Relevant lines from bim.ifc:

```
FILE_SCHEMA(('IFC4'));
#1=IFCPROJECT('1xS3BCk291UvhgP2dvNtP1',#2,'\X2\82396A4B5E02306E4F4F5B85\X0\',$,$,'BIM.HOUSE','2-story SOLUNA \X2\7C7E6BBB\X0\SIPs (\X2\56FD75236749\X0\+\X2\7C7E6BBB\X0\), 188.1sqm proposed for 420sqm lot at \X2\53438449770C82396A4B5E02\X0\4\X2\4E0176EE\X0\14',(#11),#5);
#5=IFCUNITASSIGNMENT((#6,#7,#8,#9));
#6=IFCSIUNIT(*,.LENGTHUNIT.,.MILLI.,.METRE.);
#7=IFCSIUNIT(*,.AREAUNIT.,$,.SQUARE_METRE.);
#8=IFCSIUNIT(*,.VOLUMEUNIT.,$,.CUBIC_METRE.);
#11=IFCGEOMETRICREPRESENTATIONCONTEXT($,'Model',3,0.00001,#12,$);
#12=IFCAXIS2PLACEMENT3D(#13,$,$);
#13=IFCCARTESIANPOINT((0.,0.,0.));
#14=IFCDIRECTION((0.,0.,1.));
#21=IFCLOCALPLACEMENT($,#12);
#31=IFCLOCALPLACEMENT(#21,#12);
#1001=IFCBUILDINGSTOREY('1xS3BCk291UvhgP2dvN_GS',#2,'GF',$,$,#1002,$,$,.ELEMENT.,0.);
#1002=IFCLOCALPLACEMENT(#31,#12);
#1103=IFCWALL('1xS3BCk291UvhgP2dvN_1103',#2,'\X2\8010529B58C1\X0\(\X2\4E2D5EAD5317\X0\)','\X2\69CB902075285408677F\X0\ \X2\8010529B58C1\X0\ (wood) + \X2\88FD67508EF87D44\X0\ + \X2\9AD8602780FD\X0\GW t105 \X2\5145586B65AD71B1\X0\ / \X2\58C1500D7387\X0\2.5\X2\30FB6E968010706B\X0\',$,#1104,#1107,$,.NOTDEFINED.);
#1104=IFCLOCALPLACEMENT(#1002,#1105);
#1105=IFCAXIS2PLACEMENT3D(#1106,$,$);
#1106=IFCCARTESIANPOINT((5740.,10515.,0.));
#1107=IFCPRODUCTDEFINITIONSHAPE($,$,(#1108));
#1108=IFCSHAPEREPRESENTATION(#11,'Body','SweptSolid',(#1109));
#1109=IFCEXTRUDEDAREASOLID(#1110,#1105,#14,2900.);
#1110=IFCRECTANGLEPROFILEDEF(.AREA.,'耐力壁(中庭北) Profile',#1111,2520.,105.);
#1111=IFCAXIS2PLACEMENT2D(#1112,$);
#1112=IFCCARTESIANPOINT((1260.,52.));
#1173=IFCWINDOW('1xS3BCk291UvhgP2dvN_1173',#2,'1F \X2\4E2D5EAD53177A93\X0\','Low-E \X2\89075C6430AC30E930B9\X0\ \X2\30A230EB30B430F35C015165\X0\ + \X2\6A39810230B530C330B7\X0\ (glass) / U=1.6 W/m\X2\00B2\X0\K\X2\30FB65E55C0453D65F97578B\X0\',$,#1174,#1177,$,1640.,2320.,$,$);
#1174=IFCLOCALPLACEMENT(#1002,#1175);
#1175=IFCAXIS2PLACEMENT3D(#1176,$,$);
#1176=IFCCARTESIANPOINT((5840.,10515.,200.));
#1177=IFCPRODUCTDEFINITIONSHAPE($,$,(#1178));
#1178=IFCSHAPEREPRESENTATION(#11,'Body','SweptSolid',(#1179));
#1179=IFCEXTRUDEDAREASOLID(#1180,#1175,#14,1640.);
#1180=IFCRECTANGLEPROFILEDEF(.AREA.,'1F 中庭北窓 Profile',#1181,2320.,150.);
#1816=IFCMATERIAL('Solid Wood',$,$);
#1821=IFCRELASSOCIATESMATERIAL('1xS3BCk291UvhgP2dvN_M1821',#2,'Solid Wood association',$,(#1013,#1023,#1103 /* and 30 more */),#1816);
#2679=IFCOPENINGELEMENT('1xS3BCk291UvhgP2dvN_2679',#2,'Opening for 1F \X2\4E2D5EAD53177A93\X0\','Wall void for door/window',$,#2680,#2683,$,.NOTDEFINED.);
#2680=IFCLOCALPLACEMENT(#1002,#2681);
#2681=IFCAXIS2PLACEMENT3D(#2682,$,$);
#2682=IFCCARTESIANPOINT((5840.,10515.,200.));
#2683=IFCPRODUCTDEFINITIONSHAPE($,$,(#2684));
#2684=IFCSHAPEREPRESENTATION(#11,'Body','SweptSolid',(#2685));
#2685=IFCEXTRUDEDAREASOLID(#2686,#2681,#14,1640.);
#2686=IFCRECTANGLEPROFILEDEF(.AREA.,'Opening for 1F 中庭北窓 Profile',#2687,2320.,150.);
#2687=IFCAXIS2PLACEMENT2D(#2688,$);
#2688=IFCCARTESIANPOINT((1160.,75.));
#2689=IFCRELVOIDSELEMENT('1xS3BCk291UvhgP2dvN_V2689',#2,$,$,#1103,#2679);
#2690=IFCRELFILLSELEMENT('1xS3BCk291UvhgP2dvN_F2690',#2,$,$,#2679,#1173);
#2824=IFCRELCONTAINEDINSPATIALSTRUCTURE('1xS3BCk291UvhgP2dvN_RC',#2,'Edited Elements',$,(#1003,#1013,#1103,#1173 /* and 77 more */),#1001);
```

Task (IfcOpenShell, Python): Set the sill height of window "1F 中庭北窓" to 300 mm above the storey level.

```python
import numpy as np
import ifcopenshell
import ifcopenshell.api.geometry
import ifcopenshell.geom
import ifcopenshell.util.element
import ifcopenshell.util.placement
import ifcopenshell.util.shape
import ifcopenshell.util.unit

model = ifcopenshell.open("bim.ifc")
unit_scale = ifcopenshell.util.unit.calculate_unit_scale(model)

window = model.by_guid("1xS3BCk291UvhgP2dvN_1173")
opening = window.FillsVoids[0].RelatingOpeningElement
storey = ifcopenshell.util.element.get_container(window, ifc_class="IfcBuildingStorey")
level = ifcopenshell.util.placement.get_local_placement(storey.ObjectPlacement)[2, 3]

# The opening's origin need not be at the sill, so measure its lowest point.
shape = ifcopenshell.geom.create_shape(ifcopenshell.geom.settings(), opening)
bottom = ifcopenshell.util.shape.get_shape_bottom_elevation(shape, shape.geometry) / unit_scale
dz = level + 300.0 - bottom

shift = np.array([0.0, 0.0, dz])
# The window is not placed relative to its opening, so move both.
for product in (opening, window):
    matrix = ifcopenshell.util.placement.get_local_placement(product.ObjectPlacement)
    matrix[:3, 3] += shift
    ifcopenshell.api.geometry.edit_object_placement(model, product=product, matrix=matrix, is_si=False)

print(f"moved by {dz * unit_scale:+.3f} m")

model.write("bim_updated.ifc")
```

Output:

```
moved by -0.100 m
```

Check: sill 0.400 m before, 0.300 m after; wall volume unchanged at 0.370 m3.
